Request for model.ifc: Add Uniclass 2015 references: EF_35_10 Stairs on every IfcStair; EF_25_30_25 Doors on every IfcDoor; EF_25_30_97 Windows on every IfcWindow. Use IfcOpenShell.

First a look at what the model holds.

```python
import ifcopenshell

model = ifcopenshell.open("model.ifc")
print(model.schema)
print("classifications:", [c.Name for c in model.by_type("IfcClassification")])
for ifc_class in ("IfcDoor", "IfcRoof", "IfcStair", "IfcWall", "IfcWindow"):
    print(ifc_class, len(model.by_type(ifc_class)))
```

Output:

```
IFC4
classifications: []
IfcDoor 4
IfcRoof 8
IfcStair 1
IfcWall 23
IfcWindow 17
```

```python
import ifcopenshell
import ifcopenshell.api.classification

model = ifcopenshell.open("model.ifc")

system = ifcopenshell.api.classification.add_classification(model, classification="Uniclass 2015")

codes = {
    "IfcStair": ("EF_35_10", "Stairs"),
    "IfcDoor": ("EF_25_30_25", "Doors"),
    "IfcWindow": ("EF_25_30_97", "Windows"),
}
for ifc_class, (code, name) in codes.items():
    products = model.by_type(ifc_class)
    ifcopenshell.api.classification.add_reference(
        model, products=products, classification=system, identification=code, name=name
    )
    print(code, len(products))

model.write("model-out.ifc")
```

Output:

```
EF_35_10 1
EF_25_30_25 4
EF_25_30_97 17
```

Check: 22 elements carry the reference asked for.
